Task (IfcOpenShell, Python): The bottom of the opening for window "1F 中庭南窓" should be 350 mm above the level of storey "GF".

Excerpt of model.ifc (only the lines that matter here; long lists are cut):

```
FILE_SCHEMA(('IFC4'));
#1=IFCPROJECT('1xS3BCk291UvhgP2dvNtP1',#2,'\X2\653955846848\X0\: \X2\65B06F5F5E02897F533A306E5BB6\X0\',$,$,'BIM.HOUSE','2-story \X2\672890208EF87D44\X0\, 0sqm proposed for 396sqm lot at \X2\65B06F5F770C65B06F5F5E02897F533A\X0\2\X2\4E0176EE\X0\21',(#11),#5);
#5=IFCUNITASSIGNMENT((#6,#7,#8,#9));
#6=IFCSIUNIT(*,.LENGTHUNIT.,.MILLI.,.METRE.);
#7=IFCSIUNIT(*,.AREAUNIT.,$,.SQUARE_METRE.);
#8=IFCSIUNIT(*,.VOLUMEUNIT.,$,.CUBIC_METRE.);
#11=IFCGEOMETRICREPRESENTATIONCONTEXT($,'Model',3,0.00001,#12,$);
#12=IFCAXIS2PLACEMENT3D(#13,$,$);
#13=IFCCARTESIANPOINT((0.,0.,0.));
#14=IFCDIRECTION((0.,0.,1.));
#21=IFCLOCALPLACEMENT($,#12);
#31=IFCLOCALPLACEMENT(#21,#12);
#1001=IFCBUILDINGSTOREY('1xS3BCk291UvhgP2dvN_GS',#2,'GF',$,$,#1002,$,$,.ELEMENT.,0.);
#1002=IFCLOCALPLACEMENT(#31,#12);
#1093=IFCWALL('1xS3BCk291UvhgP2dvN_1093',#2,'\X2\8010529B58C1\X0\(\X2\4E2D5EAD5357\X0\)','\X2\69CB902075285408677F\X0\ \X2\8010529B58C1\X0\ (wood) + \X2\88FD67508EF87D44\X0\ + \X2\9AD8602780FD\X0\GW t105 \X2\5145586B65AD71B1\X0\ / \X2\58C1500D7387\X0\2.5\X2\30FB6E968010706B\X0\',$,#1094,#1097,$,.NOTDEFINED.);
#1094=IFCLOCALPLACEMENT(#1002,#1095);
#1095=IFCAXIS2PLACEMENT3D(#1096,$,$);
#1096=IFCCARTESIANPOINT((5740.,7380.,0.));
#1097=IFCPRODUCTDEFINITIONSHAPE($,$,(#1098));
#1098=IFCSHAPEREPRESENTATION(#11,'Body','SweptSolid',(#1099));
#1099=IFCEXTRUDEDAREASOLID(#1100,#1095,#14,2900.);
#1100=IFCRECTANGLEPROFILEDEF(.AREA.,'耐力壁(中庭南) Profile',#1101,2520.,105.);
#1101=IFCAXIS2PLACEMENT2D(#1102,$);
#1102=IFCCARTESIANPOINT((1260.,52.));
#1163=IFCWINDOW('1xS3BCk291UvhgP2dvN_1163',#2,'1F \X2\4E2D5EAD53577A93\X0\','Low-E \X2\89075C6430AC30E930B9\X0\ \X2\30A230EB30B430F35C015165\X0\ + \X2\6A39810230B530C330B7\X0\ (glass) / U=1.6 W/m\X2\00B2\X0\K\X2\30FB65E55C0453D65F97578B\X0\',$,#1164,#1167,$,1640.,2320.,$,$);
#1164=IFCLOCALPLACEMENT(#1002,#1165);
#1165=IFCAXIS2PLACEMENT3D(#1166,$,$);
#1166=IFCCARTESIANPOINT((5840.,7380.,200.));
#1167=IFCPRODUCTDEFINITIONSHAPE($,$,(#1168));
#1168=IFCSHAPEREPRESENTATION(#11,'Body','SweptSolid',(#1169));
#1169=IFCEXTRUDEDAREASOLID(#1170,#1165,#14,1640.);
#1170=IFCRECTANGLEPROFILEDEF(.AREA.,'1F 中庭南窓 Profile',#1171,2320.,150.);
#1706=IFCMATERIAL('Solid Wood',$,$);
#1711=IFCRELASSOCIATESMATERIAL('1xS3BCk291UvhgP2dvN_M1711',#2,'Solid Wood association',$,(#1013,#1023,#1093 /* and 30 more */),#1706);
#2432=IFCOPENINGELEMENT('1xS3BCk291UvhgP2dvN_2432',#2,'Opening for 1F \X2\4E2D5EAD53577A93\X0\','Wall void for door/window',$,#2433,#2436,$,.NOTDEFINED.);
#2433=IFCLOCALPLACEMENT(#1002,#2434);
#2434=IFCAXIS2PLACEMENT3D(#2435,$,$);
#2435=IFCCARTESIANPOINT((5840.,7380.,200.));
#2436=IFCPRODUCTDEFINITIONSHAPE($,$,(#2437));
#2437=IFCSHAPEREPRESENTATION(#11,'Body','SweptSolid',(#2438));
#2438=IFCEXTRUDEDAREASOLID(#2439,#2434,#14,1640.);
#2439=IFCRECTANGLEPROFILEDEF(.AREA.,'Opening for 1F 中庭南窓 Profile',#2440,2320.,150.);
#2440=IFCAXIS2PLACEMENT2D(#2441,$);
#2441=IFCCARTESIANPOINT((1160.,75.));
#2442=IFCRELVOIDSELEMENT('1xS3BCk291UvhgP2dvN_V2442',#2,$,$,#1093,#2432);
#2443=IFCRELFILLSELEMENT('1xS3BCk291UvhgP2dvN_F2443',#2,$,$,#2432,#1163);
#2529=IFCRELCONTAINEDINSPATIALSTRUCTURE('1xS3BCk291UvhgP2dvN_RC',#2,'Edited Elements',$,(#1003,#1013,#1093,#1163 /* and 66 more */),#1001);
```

```python
import numpy as np
import ifcopenshell
import ifcopenshell.api.geometry
import ifcopenshell.geom
import ifcopenshell.util.element
import ifcopenshell.util.placement
import ifcopenshell.util.shape
import ifcopenshell.util.unit

model = ifcopenshell.open("model.ifc")
unit_scale = ifcopenshell.util.unit.calculate_unit_scale(model)

window = model.by_guid("1xS3BCk291UvhgP2dvN_1163")
opening = window.FillsVoids[0].RelatingOpeningElement
storey = ifcopenshell.util.element.get_container(window, ifc_class="IfcBuildingStorey")
level = ifcopenshell.util.placement.get_local_placement(storey.ObjectPlacement)[2, 3]

# The opening's origin need not be at the sill, so measure its lowest point.
shape = ifcopenshell.geom.create_shape(ifcopenshell.geom.settings(), opening)
bottom = ifcopenshell.util.shape.get_shape_bottom_elevation(shape, shape.geometry) / unit_scale
dz = level + 350.0 - bottom

shift = np.array([0.0, 0.0, dz])
# The window is not placed relative to its opening, so move both.
for product in (opening, window):
    matrix = ifcopenshell.util.placement.get_local_placement(product.ObjectPlacement)
    matrix[:3, 3] += shift
    ifcopenshell.api.geometry.edit_object_placement(model, product=product, matrix=matrix, is_si=False)

print(f"moved by {dz * unit_scale:+.3f} m")

model.write("model_rev.ifc")
```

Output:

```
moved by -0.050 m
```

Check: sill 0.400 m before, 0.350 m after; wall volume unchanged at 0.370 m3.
